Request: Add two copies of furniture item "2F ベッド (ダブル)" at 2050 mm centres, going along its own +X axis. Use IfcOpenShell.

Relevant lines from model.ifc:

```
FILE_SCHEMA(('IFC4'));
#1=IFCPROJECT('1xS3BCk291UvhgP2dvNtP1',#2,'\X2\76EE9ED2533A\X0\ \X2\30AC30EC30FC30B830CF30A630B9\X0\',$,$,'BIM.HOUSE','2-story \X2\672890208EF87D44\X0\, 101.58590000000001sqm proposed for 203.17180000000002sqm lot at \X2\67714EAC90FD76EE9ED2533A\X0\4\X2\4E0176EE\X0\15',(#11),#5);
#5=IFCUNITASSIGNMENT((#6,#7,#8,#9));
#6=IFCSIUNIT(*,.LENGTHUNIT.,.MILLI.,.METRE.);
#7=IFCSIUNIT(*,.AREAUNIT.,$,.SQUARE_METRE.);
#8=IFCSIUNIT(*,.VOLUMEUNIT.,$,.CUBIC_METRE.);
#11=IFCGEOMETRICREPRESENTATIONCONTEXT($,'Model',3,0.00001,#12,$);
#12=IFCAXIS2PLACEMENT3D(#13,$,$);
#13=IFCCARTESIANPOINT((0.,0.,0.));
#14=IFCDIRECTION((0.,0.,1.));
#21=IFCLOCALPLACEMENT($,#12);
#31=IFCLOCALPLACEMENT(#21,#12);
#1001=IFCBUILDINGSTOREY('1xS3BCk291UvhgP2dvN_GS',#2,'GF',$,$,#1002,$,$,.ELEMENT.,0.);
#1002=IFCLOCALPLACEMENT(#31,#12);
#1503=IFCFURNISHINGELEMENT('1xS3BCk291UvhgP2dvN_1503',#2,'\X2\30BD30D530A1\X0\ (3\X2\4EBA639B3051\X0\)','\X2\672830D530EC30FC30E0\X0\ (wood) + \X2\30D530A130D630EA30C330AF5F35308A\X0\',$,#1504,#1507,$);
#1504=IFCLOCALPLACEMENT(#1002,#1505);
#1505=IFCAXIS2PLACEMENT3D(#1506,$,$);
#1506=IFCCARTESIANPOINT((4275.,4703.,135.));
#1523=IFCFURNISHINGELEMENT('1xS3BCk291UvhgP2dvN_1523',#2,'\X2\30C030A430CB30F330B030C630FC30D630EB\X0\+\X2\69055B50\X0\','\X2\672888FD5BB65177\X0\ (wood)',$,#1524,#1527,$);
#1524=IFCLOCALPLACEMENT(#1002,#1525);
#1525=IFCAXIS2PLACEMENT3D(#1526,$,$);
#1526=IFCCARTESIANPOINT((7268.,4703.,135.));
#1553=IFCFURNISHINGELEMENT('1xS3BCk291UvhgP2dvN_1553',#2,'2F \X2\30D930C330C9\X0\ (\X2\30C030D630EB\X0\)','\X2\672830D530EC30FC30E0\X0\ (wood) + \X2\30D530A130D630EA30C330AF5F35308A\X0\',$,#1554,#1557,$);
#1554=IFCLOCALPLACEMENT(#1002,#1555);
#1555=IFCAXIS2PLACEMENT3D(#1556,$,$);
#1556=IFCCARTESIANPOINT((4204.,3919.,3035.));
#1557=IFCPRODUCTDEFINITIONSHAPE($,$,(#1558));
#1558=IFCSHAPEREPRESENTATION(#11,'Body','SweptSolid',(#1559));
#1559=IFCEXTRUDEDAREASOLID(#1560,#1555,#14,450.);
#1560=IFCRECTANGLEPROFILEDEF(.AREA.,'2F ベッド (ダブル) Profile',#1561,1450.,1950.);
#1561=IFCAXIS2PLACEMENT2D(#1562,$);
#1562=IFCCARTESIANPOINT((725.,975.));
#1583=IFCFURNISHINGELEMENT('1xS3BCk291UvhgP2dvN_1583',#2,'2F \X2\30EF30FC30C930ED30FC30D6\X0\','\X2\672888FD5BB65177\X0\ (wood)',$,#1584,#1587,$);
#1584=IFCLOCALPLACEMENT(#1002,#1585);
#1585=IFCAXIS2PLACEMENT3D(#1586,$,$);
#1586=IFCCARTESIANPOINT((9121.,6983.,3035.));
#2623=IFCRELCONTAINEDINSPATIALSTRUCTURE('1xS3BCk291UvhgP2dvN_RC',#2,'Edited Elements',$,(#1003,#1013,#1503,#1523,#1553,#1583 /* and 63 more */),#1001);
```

```python
import ifcopenshell
import ifcopenshell.api.geometry
import ifcopenshell.api.root
import ifcopenshell.util.element
import ifcopenshell.util.placement

model = ifcopenshell.open("model.ifc")


def reuse_history(source, copy):
    """copy_class also copies each property set's owner history, people and application; keep the originals."""
    for rel in copy.IsDefinedBy:
        if rel.is_a("IfcRelDefinesByProperties") and (history := rel.RelatingPropertyDefinition.OwnerHistory):
            rel.RelatingPropertyDefinition.OwnerHistory = source.OwnerHistory
            ifcopenshell.util.element.remove_deep2(model, history)


source = model.by_guid("1xS3BCk291UvhgP2dvN_1553")
base = ifcopenshell.util.placement.get_local_placement(source.ObjectPlacement)
step = base[:3, 0] * 2050.0

for i in range(1, 3):
    copy = ifcopenshell.api.root.copy_class(model, product=source)
    copy.Representation = ifcopenshell.util.element.copy_deep(
        model, source.Representation, exclude=["IfcGeometricRepresentationContext", "IfcRepresentationMap"]
    )
    reuse_history(source, copy)
    matrix = base.copy()
    matrix[:3, 3] += i * step
    print("added at", matrix[:3, 3].round(3) + 0.0)
    ifcopenshell.api.geometry.edit_object_placement(model, product=copy, matrix=matrix, is_si=False)

model.write("model_edited.ifc")
```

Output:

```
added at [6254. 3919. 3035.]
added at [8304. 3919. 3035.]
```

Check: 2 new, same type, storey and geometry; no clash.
